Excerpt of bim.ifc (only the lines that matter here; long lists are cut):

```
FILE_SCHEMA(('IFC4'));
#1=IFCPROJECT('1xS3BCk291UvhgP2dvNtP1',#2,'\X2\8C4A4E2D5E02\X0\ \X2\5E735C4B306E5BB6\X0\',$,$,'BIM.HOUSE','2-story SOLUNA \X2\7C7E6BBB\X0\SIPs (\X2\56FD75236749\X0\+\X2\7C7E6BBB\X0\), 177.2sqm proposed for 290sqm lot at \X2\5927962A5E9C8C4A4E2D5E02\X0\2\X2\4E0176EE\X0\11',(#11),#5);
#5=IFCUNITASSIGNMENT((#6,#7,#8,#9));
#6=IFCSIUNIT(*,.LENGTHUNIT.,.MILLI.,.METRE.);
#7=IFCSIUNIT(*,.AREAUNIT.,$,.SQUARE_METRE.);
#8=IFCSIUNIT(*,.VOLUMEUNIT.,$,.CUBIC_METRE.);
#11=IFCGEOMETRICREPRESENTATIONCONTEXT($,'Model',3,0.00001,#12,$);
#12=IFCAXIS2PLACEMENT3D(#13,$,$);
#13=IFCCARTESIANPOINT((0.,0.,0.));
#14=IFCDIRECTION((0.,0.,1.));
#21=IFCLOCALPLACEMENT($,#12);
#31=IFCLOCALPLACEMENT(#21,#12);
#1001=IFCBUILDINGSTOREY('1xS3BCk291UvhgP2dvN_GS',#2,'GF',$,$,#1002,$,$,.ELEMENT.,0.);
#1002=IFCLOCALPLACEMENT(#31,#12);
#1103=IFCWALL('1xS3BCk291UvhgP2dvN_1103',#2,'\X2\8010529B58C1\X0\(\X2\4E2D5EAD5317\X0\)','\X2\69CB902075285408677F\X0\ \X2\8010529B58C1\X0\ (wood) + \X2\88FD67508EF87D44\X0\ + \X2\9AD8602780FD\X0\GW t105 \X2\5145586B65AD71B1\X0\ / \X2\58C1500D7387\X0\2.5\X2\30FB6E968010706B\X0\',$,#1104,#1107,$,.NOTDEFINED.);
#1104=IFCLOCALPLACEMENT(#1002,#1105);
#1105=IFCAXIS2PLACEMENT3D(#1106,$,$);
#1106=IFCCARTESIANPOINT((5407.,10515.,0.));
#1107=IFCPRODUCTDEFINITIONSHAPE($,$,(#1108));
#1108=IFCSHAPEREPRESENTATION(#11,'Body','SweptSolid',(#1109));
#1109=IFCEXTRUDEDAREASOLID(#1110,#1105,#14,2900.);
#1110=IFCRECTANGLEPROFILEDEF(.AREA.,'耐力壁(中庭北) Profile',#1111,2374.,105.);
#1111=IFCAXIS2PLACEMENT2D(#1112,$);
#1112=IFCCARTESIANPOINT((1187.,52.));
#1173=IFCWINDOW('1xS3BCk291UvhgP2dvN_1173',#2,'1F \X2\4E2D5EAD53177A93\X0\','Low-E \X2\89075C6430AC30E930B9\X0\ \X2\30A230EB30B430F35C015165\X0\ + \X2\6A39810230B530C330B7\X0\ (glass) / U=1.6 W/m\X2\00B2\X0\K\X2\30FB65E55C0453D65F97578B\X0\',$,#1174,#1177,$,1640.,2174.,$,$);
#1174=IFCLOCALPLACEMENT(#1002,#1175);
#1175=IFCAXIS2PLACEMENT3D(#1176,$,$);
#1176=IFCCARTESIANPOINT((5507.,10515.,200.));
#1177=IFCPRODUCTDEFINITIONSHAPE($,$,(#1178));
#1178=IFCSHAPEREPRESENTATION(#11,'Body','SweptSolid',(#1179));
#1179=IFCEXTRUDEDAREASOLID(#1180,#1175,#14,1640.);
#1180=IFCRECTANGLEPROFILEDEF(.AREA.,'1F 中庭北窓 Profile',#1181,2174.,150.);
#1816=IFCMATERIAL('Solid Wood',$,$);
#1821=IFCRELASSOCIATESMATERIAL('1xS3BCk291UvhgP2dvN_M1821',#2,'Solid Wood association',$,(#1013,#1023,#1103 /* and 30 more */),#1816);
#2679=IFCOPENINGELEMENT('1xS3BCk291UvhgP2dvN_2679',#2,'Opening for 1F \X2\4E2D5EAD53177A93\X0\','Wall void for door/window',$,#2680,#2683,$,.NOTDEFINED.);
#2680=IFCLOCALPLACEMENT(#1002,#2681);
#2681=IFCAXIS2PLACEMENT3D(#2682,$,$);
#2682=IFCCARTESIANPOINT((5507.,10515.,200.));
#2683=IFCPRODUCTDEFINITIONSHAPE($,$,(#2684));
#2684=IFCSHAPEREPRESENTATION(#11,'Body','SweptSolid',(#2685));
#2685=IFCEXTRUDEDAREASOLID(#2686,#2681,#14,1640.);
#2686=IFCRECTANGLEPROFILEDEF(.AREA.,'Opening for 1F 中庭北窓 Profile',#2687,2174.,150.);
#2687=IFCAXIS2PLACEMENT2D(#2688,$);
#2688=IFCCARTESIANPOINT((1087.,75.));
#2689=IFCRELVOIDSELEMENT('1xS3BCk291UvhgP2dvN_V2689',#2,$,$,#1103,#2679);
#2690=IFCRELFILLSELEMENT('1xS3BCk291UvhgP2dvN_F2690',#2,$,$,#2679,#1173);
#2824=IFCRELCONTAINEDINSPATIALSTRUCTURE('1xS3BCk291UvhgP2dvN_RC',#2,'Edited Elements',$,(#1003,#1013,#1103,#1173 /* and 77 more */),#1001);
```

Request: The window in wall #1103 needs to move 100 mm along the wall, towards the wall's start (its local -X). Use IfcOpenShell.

```python
import ifcopenshell
import ifcopenshell.api.geometry
import ifcopenshell.util.placement
import ifcopenshell.util.unit

model = ifcopenshell.open("bim.ifc")
unit_scale = ifcopenshell.util.unit.calculate_unit_scale(model)

window = model.by_guid("1xS3BCk291UvhgP2dvN_1173")
opening = window.FillsVoids[0].RelatingOpeningElement
wall = opening.VoidsElements[0].RelatingBuildingElement

wall_matrix = ifcopenshell.util.placement.get_local_placement(wall.ObjectPlacement)
shift = wall_matrix[:3, 0] * -0.1 / unit_scale
before = ifcopenshell.util.placement.get_local_placement(window.ObjectPlacement)[:3, 3].copy()

# The window is not placed relative to its opening, so move both.
for product in (opening, window):
    matrix = ifcopenshell.util.placement.get_local_placement(product.ObjectPlacement)
    matrix[:3, 3] += shift
    ifcopenshell.api.geometry.edit_object_placement(model, product=product, matrix=matrix, is_si=False)

after = ifcopenshell.util.placement.get_local_placement(window.ObjectPlacement)[:3, 3]
print("window moved by", (after - before).round(3) + 0.0)

model.write("bim_updated.ifc")
```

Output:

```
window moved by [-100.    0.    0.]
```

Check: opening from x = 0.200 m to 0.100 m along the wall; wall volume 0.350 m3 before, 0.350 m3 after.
